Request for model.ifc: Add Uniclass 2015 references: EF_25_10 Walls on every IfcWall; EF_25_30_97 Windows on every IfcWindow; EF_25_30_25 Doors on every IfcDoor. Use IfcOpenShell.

First a look at what the model holds.

```python
import ifcopenshell

model = ifcopenshell.open("model.ifc")
print(model.schema)
print("classifications:", [c.Name for c in model.by_type("IfcClassification")])
for ifc_class in ("IfcDoor", "IfcRoof", "IfcStair", "IfcWall", "IfcWindow"):
    print(ifc_class, len(model.by_type(ifc_class)))
```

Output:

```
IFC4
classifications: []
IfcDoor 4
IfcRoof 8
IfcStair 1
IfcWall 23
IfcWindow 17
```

```python
import ifcopenshell
import ifcopenshell.api.classification

model = ifcopenshell.open("model.ifc")

system = ifcopenshell.api.classification.add_classification(model, classification="Uniclass 2015")

codes = {
    "IfcWall": ("EF_25_10", "Walls"),
    "IfcWindow": ("EF_25_30_97", "Windows"),
    "IfcDoor": ("EF_25_30_25", "Doors"),
}
for ifc_class, (code, name) in codes.items():
    products = model.by_type(ifc_class)
    ifcopenshell.api.classification.add_reference(
        model, products=products, classification=system, identification=code, name=name
    )
    print(code, len(products))

model.write("model_v2.ifc")
```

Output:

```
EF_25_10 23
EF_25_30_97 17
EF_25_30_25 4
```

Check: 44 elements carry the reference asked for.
